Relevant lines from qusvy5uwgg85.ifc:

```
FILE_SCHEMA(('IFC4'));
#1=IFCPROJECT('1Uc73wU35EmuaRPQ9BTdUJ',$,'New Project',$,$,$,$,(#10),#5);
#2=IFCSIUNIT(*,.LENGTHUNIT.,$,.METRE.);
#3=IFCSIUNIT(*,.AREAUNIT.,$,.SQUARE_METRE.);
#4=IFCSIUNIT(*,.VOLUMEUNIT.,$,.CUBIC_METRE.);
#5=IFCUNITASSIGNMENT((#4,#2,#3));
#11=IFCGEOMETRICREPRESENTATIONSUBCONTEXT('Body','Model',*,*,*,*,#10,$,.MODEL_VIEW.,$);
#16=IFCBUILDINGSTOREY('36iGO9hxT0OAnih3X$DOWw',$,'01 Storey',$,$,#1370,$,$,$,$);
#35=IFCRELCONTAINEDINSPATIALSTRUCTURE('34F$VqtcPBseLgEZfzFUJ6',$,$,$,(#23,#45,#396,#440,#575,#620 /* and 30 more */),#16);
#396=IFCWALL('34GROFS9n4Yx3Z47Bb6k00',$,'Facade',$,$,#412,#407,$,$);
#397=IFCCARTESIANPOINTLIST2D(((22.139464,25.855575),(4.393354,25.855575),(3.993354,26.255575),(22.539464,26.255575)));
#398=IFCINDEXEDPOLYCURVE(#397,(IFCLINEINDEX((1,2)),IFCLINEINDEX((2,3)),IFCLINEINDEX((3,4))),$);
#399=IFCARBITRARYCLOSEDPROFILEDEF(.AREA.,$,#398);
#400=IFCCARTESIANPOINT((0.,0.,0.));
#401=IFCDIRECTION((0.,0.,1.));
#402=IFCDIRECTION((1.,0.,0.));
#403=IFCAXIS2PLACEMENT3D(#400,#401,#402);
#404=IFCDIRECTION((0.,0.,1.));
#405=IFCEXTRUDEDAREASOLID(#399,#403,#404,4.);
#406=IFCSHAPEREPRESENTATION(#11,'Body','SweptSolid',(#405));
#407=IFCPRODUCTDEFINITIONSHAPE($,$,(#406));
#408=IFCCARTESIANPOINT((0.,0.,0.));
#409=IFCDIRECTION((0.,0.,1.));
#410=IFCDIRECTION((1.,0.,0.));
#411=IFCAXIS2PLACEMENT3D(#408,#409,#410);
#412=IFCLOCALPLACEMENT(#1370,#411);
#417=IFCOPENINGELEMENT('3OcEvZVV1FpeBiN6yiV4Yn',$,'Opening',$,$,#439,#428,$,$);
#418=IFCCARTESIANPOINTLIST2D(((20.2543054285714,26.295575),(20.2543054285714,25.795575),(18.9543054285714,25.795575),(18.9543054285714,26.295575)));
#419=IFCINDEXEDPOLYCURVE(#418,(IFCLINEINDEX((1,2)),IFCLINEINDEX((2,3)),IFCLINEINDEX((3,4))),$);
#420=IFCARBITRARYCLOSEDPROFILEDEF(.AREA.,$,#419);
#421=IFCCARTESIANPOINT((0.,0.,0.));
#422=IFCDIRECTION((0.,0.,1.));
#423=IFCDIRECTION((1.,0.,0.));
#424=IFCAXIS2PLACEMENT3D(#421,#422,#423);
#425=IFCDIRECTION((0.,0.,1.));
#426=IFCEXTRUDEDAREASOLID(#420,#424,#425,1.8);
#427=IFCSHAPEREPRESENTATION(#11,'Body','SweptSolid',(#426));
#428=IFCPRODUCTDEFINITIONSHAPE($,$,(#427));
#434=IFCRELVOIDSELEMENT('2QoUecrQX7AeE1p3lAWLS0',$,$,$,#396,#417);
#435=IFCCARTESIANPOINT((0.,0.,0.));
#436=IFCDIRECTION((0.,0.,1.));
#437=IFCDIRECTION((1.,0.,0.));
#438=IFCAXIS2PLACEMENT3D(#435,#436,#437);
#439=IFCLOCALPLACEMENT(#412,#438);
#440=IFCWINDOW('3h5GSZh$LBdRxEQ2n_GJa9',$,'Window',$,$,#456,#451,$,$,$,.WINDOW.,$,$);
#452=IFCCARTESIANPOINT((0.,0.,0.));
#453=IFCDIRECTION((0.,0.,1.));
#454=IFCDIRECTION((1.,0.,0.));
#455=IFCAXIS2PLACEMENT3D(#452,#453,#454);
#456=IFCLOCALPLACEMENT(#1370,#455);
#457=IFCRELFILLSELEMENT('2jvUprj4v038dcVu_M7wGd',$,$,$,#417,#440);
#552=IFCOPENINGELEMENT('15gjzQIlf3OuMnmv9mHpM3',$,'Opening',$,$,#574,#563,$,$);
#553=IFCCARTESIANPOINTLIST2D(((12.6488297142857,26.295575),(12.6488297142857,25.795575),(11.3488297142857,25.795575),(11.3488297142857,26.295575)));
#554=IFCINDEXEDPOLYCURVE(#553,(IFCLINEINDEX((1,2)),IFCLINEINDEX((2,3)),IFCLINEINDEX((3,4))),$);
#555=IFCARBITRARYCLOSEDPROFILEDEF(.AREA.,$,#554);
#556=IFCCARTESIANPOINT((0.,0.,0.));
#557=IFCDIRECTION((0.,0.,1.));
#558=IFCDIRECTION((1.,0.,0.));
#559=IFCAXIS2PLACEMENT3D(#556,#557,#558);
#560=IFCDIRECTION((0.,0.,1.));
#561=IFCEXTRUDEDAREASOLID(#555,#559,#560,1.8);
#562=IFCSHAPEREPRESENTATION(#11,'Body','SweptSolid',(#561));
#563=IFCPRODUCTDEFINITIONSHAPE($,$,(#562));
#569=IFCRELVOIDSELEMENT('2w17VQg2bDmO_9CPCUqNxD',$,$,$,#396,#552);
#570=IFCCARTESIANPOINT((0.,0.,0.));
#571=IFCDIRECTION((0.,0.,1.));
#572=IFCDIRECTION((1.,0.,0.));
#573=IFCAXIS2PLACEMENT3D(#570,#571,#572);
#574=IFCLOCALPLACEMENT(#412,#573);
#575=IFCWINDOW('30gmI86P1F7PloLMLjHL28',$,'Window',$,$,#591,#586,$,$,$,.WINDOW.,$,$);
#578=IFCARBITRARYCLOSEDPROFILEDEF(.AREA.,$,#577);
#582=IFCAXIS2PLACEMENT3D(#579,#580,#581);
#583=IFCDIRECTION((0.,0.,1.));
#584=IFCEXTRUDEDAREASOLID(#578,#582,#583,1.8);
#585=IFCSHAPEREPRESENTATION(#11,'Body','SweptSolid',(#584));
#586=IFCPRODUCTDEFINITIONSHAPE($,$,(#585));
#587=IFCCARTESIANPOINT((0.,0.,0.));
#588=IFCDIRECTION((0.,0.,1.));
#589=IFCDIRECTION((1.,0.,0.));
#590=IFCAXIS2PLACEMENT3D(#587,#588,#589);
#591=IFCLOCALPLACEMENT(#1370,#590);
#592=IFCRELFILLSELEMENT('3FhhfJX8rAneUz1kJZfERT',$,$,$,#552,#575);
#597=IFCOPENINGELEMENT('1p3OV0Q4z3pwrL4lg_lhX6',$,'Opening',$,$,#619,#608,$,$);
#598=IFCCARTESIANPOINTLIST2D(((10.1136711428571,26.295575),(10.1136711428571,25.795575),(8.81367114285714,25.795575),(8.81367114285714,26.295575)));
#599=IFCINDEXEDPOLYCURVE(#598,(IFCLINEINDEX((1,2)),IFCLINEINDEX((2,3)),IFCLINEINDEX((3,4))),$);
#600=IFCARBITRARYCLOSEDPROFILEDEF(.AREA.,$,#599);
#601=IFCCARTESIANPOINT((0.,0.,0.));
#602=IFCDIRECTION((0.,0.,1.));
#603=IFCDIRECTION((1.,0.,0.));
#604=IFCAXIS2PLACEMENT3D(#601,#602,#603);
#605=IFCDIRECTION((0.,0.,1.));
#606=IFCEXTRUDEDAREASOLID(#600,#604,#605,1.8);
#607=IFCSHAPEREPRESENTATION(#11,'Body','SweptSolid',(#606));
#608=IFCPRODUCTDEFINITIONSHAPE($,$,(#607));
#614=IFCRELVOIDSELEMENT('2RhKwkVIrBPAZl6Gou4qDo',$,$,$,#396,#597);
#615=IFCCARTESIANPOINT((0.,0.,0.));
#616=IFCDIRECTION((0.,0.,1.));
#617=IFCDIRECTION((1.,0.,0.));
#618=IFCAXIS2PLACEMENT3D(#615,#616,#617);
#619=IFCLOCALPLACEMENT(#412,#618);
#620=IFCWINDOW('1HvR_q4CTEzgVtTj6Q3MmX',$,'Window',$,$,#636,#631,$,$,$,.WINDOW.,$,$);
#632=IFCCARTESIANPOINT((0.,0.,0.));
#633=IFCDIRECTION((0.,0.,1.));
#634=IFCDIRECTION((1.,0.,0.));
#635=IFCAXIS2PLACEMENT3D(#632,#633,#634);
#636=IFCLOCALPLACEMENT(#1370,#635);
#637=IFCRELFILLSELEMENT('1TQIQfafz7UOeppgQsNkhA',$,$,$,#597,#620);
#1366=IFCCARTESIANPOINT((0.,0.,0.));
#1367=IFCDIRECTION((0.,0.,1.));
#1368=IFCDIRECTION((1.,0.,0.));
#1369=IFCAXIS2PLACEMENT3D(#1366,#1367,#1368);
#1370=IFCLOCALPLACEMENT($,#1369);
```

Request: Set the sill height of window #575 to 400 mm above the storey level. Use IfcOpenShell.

```python
import numpy as np
import ifcopenshell
import ifcopenshell.api.geometry
import ifcopenshell.geom
import ifcopenshell.util.element
import ifcopenshell.util.placement
import ifcopenshell.util.shape
import ifcopenshell.util.unit

model = ifcopenshell.open("qusvy5uwgg85.ifc")
unit_scale = ifcopenshell.util.unit.calculate_unit_scale(model)

window = model.by_id(575)
opening = window.FillsVoids[0].RelatingOpeningElement
storey = ifcopenshell.util.element.get_container(window, ifc_class="IfcBuildingStorey")
level = ifcopenshell.util.placement.get_local_placement(storey.ObjectPlacement)[2, 3]

# The opening's origin need not be at the sill, so measure its lowest point.
shape = ifcopenshell.geom.create_shape(ifcopenshell.geom.settings(), opening)
bottom = ifcopenshell.util.shape.get_shape_bottom_elevation(shape, shape.geometry) / unit_scale
dz = level + 0.4 / unit_scale - bottom

shift = np.array([0.0, 0.0, dz])
# The window is not placed relative to its opening, so move both.
for product in (opening, window):
    matrix = ifcopenshell.util.placement.get_local_placement(product.ObjectPlacement)
    matrix[:3, 3] += shift
    ifcopenshell.api.geometry.edit_object_placement(model, product=product, matrix=matrix, is_si=False)

print(f"moved by {dz * unit_scale:+.3f} m")

model.write("qusvy5uwgg85_edited.ifc")
```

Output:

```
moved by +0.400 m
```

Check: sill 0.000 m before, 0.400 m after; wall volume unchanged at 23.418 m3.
